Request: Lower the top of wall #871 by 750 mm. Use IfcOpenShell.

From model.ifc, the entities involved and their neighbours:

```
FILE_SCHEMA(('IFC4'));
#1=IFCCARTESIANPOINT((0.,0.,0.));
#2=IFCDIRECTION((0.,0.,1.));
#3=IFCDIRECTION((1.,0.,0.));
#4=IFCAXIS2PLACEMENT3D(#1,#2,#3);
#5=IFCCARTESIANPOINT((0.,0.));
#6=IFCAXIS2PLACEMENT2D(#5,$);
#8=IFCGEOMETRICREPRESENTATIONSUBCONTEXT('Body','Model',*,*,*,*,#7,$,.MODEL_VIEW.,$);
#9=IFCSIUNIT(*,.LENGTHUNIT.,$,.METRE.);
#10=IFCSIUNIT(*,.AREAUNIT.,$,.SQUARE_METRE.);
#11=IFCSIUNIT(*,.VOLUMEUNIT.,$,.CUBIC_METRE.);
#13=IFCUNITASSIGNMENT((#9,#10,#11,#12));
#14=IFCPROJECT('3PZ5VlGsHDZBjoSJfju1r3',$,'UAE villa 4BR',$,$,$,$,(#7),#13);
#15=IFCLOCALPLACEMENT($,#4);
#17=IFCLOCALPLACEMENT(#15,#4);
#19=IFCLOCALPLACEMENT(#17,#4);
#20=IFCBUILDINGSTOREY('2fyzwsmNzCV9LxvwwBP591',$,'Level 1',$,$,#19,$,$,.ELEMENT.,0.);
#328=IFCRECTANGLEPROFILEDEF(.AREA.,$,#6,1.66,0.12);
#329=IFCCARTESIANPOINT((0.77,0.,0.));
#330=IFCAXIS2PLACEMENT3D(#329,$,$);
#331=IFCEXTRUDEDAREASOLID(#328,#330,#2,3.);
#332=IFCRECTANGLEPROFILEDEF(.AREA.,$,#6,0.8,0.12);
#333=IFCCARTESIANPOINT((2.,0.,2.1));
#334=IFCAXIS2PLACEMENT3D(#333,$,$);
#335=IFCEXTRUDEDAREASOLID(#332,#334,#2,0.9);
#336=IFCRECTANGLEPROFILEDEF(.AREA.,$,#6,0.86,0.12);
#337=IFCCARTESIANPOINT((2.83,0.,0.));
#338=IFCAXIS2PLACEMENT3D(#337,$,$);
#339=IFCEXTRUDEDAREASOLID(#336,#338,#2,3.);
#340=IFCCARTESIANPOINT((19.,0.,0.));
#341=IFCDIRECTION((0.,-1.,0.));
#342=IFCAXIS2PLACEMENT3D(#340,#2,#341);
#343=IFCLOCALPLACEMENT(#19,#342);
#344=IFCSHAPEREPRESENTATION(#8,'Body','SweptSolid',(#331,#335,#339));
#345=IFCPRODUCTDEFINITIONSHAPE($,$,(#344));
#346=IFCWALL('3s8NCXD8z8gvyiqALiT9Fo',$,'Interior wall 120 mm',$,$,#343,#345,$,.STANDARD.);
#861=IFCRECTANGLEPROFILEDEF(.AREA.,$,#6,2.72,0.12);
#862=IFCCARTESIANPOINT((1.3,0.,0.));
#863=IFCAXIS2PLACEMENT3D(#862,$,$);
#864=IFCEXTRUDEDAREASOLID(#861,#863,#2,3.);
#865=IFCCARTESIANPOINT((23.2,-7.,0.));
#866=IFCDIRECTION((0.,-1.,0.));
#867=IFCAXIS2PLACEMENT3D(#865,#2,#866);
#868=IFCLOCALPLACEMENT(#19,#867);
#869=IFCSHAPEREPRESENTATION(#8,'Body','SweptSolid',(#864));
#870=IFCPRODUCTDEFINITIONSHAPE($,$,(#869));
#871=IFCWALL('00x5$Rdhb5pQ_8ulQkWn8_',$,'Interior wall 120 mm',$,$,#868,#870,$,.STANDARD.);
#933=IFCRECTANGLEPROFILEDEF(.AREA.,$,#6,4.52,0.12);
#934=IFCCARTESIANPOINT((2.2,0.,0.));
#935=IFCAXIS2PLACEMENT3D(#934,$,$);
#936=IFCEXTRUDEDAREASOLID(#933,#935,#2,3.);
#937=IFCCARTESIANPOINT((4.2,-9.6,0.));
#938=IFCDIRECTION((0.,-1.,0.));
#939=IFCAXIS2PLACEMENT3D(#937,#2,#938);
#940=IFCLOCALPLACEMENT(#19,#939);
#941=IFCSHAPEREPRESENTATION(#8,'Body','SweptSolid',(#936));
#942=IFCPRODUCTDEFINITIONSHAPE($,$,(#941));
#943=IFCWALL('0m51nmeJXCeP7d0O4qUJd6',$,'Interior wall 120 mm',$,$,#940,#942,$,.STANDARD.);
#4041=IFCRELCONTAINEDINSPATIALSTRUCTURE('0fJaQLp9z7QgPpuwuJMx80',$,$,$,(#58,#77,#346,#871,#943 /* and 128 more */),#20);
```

```python
import ifcopenshell
import ifcopenshell.geom
import ifcopenshell.util.representation
import ifcopenshell.util.shape
import ifcopenshell.util.unit

model = ifcopenshell.open("model.ifc")
unit_scale = ifcopenshell.util.unit.calculate_unit_scale(model)
settings = ifcopenshell.geom.settings()


def volume(element):
    """Net volume in cubic metres, openings subtracted."""
    shape = ifcopenshell.geom.create_shape(settings, element)
    return ifcopenshell.util.shape.get_volume(shape.geometry)


wall = model.by_id(871)
before = volume(wall)

body = ifcopenshell.util.representation.get_representation(wall, "Model", "Body")
solid = body.Items[0]
old_height = solid.Depth
solid.Depth -= 0.75 / unit_scale
after = volume(wall)

print(f"height {old_height:g} -> {solid.Depth:g}, volume {before:.3f} -> {after:.3f} m3")

model.write("model_rev.ifc")
```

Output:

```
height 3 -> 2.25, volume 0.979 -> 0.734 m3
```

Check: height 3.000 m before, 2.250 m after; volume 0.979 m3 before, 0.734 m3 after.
